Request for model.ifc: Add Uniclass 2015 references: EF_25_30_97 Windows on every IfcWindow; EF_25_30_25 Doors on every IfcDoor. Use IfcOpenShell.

First a look at what the model holds.

```python
import ifcopenshell

model = ifcopenshell.open("model.ifc")
print(model.schema)
print("classifications:", [c.Name for c in model.by_type("IfcClassification")])
for ifc_class in ("IfcDoor", "IfcRoof", "IfcStair", "IfcWall", "IfcWindow"):
    print(ifc_class, len(model.by_type(ifc_class)))
```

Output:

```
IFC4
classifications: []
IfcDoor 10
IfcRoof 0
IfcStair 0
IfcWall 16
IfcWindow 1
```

```python
import ifcopenshell
import ifcopenshell.api.classification

model = ifcopenshell.open("model.ifc")

system = ifcopenshell.api.classification.add_classification(model, classification="Uniclass 2015")

codes = {
    "IfcWindow": ("EF_25_30_97", "Windows"),
    "IfcDoor": ("EF_25_30_25", "Doors"),
}
for ifc_class, (code, name) in codes.items():
    products = model.by_type(ifc_class)
    ifcopenshell.api.classification.add_reference(
        model, products=products, classification=system, identification=code, name=name
    )
    print(code, len(products))

model.write("model_v2.ifc")
```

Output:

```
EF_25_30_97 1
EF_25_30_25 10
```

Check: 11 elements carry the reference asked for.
